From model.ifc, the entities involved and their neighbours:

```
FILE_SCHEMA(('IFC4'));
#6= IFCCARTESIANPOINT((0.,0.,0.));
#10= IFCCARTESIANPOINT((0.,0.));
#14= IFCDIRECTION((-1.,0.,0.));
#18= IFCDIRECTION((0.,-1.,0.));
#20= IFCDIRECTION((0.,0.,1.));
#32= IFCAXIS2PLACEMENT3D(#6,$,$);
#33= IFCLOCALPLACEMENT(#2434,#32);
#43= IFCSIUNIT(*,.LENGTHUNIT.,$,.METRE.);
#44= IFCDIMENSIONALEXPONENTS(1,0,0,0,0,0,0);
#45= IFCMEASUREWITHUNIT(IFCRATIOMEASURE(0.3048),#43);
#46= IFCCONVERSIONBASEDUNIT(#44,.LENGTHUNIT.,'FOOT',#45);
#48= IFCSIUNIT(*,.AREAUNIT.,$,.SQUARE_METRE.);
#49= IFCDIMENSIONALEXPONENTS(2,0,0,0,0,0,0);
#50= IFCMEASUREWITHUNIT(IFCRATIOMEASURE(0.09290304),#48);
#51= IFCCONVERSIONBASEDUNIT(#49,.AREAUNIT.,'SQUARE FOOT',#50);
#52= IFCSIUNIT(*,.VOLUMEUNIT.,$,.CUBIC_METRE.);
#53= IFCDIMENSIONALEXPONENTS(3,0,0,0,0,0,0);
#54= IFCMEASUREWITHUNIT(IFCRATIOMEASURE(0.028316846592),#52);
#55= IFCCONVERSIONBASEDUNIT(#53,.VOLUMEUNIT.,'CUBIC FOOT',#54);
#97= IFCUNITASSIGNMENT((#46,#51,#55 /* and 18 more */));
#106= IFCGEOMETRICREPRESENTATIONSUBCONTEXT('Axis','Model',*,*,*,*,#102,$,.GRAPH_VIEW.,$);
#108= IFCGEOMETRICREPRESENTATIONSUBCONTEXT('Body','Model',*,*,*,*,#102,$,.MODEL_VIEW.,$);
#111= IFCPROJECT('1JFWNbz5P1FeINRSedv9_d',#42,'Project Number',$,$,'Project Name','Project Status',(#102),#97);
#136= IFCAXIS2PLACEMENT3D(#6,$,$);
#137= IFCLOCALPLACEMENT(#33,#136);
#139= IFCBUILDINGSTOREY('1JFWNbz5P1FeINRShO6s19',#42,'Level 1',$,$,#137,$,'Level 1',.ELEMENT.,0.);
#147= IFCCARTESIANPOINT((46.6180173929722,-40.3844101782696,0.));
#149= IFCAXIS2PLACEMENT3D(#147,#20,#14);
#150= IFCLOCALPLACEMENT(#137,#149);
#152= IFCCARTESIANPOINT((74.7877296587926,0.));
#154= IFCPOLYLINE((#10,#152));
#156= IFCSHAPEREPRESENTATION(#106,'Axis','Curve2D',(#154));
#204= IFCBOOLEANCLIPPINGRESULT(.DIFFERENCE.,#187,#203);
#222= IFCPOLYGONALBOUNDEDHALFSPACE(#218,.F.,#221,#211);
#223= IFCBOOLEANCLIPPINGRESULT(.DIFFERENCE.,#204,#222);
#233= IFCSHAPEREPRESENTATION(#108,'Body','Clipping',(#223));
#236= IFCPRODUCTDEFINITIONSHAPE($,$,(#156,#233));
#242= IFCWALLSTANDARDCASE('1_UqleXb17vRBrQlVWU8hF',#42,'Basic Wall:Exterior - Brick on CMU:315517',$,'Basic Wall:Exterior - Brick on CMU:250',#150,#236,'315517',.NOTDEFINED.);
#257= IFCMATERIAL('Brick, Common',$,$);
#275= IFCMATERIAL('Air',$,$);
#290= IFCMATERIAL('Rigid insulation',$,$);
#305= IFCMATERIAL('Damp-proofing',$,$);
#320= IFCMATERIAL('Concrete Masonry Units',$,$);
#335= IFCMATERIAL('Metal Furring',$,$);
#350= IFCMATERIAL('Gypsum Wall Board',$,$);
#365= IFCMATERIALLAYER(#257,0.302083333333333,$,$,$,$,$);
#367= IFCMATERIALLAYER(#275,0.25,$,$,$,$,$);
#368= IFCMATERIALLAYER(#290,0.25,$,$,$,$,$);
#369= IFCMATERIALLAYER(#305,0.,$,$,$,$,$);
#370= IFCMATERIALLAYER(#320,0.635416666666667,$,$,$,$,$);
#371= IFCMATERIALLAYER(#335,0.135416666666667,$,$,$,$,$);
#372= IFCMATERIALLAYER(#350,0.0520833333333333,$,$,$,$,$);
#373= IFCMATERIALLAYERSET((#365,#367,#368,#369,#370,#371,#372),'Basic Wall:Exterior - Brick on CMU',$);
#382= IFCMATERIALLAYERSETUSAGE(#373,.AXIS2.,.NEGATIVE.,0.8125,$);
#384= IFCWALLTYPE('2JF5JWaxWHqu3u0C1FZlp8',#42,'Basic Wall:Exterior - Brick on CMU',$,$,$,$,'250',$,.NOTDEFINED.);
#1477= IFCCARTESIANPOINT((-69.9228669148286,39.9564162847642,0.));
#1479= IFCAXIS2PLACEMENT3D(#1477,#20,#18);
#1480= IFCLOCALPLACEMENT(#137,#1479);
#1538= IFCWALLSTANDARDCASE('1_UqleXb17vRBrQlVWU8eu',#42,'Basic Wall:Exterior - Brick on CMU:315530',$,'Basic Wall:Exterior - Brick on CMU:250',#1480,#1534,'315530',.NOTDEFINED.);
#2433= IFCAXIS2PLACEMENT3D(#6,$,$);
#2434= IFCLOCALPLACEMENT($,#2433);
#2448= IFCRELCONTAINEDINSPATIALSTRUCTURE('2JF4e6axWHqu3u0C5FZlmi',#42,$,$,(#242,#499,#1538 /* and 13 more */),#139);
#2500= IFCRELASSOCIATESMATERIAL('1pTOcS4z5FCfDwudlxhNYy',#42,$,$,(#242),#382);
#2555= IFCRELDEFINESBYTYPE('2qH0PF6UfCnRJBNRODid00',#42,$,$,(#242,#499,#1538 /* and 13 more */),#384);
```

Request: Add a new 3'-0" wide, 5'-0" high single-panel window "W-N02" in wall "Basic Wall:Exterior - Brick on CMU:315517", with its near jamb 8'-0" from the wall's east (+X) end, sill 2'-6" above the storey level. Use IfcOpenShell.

```python
import numpy as np
import ifcopenshell
import ifcopenshell.api.feature
import ifcopenshell.api.geometry
import ifcopenshell.api.root
import ifcopenshell.api.spatial
import ifcopenshell.geom
import ifcopenshell.util.element
import ifcopenshell.util.placement
import ifcopenshell.util.representation
import ifcopenshell.util.shape
import ifcopenshell.util.unit

model = ifcopenshell.open("model.ifc")
unit_scale = ifcopenshell.util.unit.calculate_unit_scale(model)
settings = ifcopenshell.geom.settings()


def volume(element):
    """Net volume in cubic metres, openings subtracted."""
    shape = ifcopenshell.geom.create_shape(settings, element)
    return ifcopenshell.util.shape.get_volume(shape.geometry)


wall = model.by_id(242)
storey = ifcopenshell.util.element.get_container(wall, ifc_class="IfcBuildingStorey")
context = ifcopenshell.util.representation.get_context(model, "Model", "Body", "MODEL_VIEW")
before = volume(wall)

width, height, from_end, sill = 0.9144, 1.524, 2.4384, 0.762  # metres

# The wall runs along its own X axis, and the end named is its -X end.
wall_shape = ifcopenshell.geom.create_shape(settings, wall)
x, y, z = ifcopenshell.util.shape.get_vertices(wall_shape.geometry).T
start = x.min() + from_end
face, thickness = float(y.min()), float(y.max() - y.min())
wall_matrix = ifcopenshell.util.placement.get_local_placement(wall.ObjectPlacement)
level = ifcopenshell.util.placement.get_local_placement(storey.ObjectPlacement)[2, 3]


def in_wall(x, y):
    """Placement at x, y metres in the wall's axes, at sill height."""
    matrix = wall_matrix.copy()
    matrix[:, 3] = wall_matrix @ np.array([x / unit_scale, y / unit_scale, 0.0, 1.0])
    matrix[2, 3] = level + sill / unit_scale
    return matrix


# Opening: a box that overshoots both wall faces by 50 mm.
opening = ifcopenshell.api.root.create_entity(model, ifc_class="IfcOpeningElement", predefined_type="OPENING")
box = ifcopenshell.api.geometry.add_wall_representation(
    model, context=context, length=width, height=height, thickness=thickness + 0.1
)
ifcopenshell.api.geometry.assign_representation(model, product=opening, representation=box)
ifcopenshell.api.geometry.edit_object_placement(model, product=opening, matrix=in_wall(start, face - 0.05), is_si=False)
ifcopenshell.api.feature.add_feature(model, feature=opening, element=wall)

window = ifcopenshell.api.root.create_entity(model, ifc_class="IfcWindow", name="W-N02", predefined_type="WINDOW")
window.OverallWidth, window.OverallHeight = width / unit_scale, height / unit_scale
window.PartitioningType = "SINGLE_PANEL"
body = ifcopenshell.api.geometry.add_window_representation(
    model,
    context=context,
    overall_width=window.OverallWidth,
    overall_height=window.OverallHeight,
    partition_type="SINGLE_PANEL",
)
ifcopenshell.api.geometry.assign_representation(model, product=window, representation=body)
ifcopenshell.api.spatial.assign_container(model, products=[window], relating_structure=storey)
ifcopenshell.api.feature.add_filling(model, opening=opening, element=window)

# Centre the window in the wall's thickness.
ifcopenshell.api.geometry.edit_object_placement(model, product=window, matrix=in_wall(start, face), is_si=False)
window_shape = ifcopenshell.geom.create_shape(settings, window)
depth = ifcopenshell.util.shape.get_vertices(window_shape.geometry)[:, 1]
offset = face + thickness / 2 - (depth.min() + depth.max()) / 2
ifcopenshell.api.geometry.edit_object_placement(model, product=window, matrix=in_wall(start, offset), is_si=False)

after = volume(wall)

print(f"wall volume {before:.3f} -> {after:.3f} m3")

model.write("model_updated.ifc")
```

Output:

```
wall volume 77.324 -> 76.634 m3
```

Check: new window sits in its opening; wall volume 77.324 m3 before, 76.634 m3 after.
